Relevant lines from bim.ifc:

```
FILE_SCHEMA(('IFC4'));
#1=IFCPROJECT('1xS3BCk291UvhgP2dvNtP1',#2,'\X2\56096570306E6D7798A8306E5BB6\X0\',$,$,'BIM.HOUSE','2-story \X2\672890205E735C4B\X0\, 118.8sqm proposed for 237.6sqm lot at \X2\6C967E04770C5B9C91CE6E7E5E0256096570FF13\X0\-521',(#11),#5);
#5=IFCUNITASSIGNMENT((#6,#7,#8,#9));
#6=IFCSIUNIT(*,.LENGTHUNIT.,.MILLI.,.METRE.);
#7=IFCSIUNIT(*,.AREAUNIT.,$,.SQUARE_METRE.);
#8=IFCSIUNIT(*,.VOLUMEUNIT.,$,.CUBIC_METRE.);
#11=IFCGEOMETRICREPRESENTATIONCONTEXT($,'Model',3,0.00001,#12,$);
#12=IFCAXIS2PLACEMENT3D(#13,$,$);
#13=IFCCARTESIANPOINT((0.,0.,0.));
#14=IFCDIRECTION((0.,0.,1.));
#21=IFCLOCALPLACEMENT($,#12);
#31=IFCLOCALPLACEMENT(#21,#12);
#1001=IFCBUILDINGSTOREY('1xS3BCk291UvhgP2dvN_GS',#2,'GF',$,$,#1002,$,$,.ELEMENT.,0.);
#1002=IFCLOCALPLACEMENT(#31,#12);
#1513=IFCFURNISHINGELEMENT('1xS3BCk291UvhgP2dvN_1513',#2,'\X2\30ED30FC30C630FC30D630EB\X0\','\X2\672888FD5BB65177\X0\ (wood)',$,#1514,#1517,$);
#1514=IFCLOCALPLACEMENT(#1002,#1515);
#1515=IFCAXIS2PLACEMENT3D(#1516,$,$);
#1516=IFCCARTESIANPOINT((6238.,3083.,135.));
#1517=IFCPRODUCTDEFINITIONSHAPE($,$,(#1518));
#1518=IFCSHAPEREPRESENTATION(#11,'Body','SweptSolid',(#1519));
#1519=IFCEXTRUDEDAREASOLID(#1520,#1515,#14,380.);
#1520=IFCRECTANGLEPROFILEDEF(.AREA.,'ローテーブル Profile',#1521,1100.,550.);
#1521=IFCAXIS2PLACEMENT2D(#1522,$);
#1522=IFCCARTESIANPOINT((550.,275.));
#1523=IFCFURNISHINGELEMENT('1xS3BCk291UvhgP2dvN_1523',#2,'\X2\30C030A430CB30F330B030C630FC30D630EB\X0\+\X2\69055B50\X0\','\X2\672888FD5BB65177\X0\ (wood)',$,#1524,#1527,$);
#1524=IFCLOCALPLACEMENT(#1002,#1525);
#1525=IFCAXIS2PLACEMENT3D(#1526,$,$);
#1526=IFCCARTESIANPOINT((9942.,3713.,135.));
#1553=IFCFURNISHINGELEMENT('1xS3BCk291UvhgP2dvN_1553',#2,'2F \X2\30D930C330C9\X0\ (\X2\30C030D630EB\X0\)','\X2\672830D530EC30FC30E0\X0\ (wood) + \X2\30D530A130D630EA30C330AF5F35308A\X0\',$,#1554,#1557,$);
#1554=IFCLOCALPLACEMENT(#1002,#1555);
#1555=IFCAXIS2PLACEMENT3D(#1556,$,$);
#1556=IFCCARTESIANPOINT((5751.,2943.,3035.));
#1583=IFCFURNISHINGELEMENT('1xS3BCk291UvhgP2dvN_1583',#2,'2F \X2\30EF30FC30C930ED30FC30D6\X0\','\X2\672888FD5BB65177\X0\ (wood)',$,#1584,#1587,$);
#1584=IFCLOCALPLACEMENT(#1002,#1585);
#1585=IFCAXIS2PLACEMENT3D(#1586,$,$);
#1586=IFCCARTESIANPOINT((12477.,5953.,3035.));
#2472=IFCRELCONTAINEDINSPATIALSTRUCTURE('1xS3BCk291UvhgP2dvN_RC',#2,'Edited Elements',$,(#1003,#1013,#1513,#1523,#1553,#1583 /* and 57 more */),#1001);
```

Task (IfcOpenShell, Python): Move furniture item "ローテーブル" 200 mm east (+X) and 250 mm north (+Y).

```python
import ifcopenshell
import ifcopenshell.api.geometry
import ifcopenshell.util.placement
import ifcopenshell.util.unit

model = ifcopenshell.open("bim.ifc")
unit_scale = ifcopenshell.util.unit.calculate_unit_scale(model)

item = model.by_guid("1xS3BCk291UvhgP2dvN_1513")
matrix = ifcopenshell.util.placement.get_local_placement(item.ObjectPlacement)
matrix[0, 3] += 0.2 / unit_scale
matrix[1, 3] += 0.25 / unit_scale
ifcopenshell.api.geometry.edit_object_placement(model, product=item, matrix=matrix, is_si=False)

print(ifcopenshell.util.placement.get_local_placement(item.ObjectPlacement).round(3) + 0.0)

model.write("bim_rev.ifc")
```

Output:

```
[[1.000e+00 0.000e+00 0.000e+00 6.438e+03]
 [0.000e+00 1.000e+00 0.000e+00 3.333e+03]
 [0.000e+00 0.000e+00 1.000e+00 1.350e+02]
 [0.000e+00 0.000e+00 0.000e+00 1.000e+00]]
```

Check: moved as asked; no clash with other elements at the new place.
